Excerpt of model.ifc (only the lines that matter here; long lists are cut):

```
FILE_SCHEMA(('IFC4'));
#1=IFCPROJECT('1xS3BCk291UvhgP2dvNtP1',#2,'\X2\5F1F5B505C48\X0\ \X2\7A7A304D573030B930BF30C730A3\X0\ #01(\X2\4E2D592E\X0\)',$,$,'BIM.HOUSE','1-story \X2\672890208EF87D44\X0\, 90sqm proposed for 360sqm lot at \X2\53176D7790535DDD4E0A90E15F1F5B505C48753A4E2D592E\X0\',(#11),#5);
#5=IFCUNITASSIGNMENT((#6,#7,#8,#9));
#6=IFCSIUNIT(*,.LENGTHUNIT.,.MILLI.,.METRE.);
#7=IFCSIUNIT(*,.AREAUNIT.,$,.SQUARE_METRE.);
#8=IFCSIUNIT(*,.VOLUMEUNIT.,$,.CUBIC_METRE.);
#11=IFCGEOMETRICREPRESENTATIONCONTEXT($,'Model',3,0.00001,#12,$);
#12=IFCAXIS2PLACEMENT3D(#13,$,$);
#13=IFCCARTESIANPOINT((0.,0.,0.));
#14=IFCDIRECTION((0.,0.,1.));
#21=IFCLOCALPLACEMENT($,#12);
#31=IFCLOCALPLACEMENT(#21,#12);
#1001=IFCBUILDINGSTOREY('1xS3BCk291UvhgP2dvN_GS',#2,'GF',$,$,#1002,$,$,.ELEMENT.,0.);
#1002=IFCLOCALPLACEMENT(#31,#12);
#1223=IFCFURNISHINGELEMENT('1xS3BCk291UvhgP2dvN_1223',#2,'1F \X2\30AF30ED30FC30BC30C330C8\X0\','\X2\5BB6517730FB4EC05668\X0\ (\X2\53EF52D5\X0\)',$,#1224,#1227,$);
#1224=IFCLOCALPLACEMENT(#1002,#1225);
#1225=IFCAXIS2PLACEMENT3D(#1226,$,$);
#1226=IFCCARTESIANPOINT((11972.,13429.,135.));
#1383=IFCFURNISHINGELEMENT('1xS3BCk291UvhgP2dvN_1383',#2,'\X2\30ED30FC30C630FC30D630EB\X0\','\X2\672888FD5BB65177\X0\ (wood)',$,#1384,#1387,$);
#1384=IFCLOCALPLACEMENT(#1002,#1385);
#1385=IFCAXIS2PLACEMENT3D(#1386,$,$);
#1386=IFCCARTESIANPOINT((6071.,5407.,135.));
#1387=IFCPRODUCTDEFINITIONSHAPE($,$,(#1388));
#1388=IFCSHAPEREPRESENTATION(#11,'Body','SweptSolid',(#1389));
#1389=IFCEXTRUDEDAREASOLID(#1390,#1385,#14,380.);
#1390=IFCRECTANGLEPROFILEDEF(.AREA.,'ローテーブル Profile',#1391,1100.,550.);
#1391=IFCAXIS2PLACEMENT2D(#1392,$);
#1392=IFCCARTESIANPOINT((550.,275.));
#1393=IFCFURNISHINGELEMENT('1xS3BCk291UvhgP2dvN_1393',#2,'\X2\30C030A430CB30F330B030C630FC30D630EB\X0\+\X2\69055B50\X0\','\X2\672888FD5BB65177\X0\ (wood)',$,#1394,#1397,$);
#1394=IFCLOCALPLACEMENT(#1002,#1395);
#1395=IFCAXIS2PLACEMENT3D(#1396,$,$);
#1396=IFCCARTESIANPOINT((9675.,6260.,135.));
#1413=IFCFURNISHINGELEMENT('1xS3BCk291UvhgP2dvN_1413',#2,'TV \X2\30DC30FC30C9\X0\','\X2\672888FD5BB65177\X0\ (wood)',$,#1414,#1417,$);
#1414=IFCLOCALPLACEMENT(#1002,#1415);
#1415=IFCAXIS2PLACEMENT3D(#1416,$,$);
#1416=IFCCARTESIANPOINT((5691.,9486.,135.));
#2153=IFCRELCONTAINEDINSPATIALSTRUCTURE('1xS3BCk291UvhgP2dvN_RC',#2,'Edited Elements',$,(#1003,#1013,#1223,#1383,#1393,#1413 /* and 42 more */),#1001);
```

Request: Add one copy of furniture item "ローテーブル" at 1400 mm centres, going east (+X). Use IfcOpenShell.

```python
import numpy as np
import ifcopenshell
import ifcopenshell.api.geometry
import ifcopenshell.api.root
import ifcopenshell.util.element
import ifcopenshell.util.placement
import ifcopenshell.util.unit

model = ifcopenshell.open("model.ifc")
unit_scale = ifcopenshell.util.unit.calculate_unit_scale(model)


def reuse_history(source, copy):
    """copy_class also copies each property set's owner history, people and application; keep the originals."""
    for rel in copy.IsDefinedBy:
        if rel.is_a("IfcRelDefinesByProperties") and (history := rel.RelatingPropertyDefinition.OwnerHistory):
            rel.RelatingPropertyDefinition.OwnerHistory = source.OwnerHistory
            ifcopenshell.util.element.remove_deep2(model, history)


source = model.by_id(1383)
base = ifcopenshell.util.placement.get_local_placement(source.ObjectPlacement)
step = np.array([1.0, 0.0, 0.0]) * 1.4 / unit_scale

for i in range(1, 2):
    copy = ifcopenshell.api.root.copy_class(model, product=source)
    copy.Representation = ifcopenshell.util.element.copy_deep(
        model, source.Representation, exclude=["IfcGeometricRepresentationContext", "IfcRepresentationMap"]
    )
    reuse_history(source, copy)
    matrix = base.copy()
    matrix[:3, 3] += i * step
    print("added at", matrix[:3, 3].round(3) + 0.0)
    ifcopenshell.api.geometry.edit_object_placement(model, product=copy, matrix=matrix, is_si=False)

model.write("model-out.ifc")
```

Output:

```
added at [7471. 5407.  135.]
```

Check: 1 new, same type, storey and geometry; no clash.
